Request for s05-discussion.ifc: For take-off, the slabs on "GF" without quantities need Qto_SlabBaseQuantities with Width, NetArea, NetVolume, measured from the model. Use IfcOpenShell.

First a look at what the model holds.

```python
import ifcopenshell
import ifcopenshell.util.element
import ifcopenshell.util.unit

model = ifcopenshell.open("s05-discussion.ifc")
print(model.schema)
for unit_type in ("LENGTHUNIT", "AREAUNIT", "VOLUMEUNIT"):
    print(unit_type, ifcopenshell.util.unit.calculate_unit_scale(model, unit_type))
storey = next(s for s in model.by_type("IfcBuildingStorey") if s.Name == "GF")
slabs = [e for e in ifcopenshell.util.element.get_decomposition(storey) if e.is_a("IfcSlab")]
for e in sorted(slabs, key=lambda e: e.id()):
    print(e.id(), e.is_a(), e.Name, list(ifcopenshell.util.element.get_psets(e, qtos_only=True)), sep=" | ")
```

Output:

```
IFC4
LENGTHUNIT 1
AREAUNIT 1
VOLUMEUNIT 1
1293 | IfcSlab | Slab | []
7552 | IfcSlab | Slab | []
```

```python
import ifcopenshell
import ifcopenshell.api.pset
import ifcopenshell.geom
import ifcopenshell.util.element
import ifcopenshell.util.shape
import ifcopenshell.util.unit

model = ifcopenshell.open("s05-discussion.ifc")
unit_scale = ifcopenshell.util.unit.calculate_unit_scale(model)
area_scale = ifcopenshell.util.unit.calculate_unit_scale(model, "AREAUNIT")
volume_scale = ifcopenshell.util.unit.calculate_unit_scale(model, "VOLUMEUNIT")
settings = ifcopenshell.geom.settings()

storey = next(s for s in model.by_type("IfcBuildingStorey") if s.Name == "GF")
slabs = [e for e in ifcopenshell.util.element.get_decomposition(storey) if e.is_a("IfcSlab")]

for e in sorted(slabs, key=lambda e: e.id()):
    if ifcopenshell.util.element.get_psets(e, qtos_only=True, should_inherit=False):
        continue
    # Geometry comes back in metres, in the element's own axes.
    shape = ifcopenshell.geom.create_shape(settings, e)
    values = {
        "Width": ifcopenshell.util.shape.get_z(shape.geometry) / unit_scale,
        "NetArea": ifcopenshell.util.shape.get_footprint_area(shape.geometry) / area_scale,
        "NetVolume": ifcopenshell.util.shape.get_volume(shape.geometry) / volume_scale,
    }
    qto = ifcopenshell.api.pset.add_qto(model, product=e, name="Qto_SlabBaseQuantities")
    ifcopenshell.api.pset.edit_qto(model, qto=qto, properties=values)
    print(e.id(), {k: round(v, 3) for k, v in values.items()})

model.write("s05-discussion-out.ifc")
```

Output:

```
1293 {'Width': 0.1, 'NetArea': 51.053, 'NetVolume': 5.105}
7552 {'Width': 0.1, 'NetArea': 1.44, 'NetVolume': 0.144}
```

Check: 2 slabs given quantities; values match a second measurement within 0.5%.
